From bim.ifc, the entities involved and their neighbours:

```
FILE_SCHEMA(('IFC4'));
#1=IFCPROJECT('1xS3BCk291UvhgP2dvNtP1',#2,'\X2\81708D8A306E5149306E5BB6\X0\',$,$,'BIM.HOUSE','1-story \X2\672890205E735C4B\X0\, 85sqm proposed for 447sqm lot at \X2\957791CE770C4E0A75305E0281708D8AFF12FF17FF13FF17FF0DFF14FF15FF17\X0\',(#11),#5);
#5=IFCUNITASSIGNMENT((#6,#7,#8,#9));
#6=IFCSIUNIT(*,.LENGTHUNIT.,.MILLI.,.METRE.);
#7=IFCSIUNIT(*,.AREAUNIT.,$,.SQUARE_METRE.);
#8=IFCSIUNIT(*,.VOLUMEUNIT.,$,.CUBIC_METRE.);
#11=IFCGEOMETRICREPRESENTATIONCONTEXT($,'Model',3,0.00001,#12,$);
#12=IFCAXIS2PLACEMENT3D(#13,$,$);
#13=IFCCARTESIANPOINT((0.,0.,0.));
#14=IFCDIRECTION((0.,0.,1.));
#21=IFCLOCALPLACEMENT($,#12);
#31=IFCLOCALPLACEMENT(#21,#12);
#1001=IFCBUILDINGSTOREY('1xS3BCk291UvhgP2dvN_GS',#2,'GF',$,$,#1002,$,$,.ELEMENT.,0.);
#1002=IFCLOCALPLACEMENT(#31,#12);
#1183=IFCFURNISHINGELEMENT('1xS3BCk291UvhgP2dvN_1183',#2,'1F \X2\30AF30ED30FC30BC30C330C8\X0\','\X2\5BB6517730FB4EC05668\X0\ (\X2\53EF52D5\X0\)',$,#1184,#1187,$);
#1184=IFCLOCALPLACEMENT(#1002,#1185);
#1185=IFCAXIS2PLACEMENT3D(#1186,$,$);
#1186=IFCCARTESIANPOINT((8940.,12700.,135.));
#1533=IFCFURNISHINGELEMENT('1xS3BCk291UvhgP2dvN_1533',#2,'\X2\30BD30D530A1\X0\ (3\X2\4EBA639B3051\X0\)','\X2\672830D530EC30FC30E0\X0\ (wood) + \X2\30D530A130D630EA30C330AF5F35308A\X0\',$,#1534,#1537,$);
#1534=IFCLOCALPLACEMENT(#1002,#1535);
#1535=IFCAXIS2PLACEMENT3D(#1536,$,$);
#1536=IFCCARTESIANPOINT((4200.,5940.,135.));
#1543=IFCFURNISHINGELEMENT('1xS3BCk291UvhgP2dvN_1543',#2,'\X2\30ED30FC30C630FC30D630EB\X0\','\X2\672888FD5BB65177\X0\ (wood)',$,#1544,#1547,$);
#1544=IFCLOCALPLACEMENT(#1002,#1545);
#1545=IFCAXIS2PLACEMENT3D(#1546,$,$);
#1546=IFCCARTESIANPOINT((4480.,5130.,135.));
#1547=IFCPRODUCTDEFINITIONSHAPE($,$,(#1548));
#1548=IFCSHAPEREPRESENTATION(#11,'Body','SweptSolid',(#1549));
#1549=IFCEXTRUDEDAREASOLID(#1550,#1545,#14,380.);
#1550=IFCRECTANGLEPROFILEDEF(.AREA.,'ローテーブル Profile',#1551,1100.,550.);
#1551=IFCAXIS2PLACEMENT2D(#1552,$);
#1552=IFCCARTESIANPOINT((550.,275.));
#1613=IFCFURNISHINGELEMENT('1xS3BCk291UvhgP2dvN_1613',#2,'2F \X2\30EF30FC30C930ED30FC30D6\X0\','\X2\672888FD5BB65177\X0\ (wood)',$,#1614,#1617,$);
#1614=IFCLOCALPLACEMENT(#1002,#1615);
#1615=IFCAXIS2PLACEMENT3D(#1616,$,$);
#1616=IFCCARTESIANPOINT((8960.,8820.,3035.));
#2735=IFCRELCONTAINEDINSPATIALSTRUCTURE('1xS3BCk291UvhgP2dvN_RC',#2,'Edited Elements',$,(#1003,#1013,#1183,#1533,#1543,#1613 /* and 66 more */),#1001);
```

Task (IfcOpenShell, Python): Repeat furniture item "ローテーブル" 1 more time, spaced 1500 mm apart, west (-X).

```python
import numpy as np
import ifcopenshell
import ifcopenshell.api.geometry
import ifcopenshell.api.root
import ifcopenshell.util.element
import ifcopenshell.util.placement
import ifcopenshell.util.unit

model = ifcopenshell.open("bim.ifc")
unit_scale = ifcopenshell.util.unit.calculate_unit_scale(model)


def reuse_history(source, copy):
    """copy_class also copies each property set's owner history, people and application; keep the originals."""
    for rel in copy.IsDefinedBy:
        if rel.is_a("IfcRelDefinesByProperties") and (history := rel.RelatingPropertyDefinition.OwnerHistory):
            rel.RelatingPropertyDefinition.OwnerHistory = source.OwnerHistory
            ifcopenshell.util.element.remove_deep2(model, history)


source = model.by_guid("1xS3BCk291UvhgP2dvN_1543")
base = ifcopenshell.util.placement.get_local_placement(source.ObjectPlacement)
step = np.array([-1.0, 0.0, 0.0]) * 1.5 / unit_scale

for i in range(1, 2):
    copy = ifcopenshell.api.root.copy_class(model, product=source)
    copy.Representation = ifcopenshell.util.element.copy_deep(
        model, source.Representation, exclude=["IfcGeometricRepresentationContext", "IfcRepresentationMap"]
    )
    reuse_history(source, copy)
    matrix = base.copy()
    matrix[:3, 3] += i * step
    print("added at", matrix[:3, 3].round(3) + 0.0)
    ifcopenshell.api.geometry.edit_object_placement(model, product=copy, matrix=matrix, is_si=False)

model.write("bim_v2.ifc")
```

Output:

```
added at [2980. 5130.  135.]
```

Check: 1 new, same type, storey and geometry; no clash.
